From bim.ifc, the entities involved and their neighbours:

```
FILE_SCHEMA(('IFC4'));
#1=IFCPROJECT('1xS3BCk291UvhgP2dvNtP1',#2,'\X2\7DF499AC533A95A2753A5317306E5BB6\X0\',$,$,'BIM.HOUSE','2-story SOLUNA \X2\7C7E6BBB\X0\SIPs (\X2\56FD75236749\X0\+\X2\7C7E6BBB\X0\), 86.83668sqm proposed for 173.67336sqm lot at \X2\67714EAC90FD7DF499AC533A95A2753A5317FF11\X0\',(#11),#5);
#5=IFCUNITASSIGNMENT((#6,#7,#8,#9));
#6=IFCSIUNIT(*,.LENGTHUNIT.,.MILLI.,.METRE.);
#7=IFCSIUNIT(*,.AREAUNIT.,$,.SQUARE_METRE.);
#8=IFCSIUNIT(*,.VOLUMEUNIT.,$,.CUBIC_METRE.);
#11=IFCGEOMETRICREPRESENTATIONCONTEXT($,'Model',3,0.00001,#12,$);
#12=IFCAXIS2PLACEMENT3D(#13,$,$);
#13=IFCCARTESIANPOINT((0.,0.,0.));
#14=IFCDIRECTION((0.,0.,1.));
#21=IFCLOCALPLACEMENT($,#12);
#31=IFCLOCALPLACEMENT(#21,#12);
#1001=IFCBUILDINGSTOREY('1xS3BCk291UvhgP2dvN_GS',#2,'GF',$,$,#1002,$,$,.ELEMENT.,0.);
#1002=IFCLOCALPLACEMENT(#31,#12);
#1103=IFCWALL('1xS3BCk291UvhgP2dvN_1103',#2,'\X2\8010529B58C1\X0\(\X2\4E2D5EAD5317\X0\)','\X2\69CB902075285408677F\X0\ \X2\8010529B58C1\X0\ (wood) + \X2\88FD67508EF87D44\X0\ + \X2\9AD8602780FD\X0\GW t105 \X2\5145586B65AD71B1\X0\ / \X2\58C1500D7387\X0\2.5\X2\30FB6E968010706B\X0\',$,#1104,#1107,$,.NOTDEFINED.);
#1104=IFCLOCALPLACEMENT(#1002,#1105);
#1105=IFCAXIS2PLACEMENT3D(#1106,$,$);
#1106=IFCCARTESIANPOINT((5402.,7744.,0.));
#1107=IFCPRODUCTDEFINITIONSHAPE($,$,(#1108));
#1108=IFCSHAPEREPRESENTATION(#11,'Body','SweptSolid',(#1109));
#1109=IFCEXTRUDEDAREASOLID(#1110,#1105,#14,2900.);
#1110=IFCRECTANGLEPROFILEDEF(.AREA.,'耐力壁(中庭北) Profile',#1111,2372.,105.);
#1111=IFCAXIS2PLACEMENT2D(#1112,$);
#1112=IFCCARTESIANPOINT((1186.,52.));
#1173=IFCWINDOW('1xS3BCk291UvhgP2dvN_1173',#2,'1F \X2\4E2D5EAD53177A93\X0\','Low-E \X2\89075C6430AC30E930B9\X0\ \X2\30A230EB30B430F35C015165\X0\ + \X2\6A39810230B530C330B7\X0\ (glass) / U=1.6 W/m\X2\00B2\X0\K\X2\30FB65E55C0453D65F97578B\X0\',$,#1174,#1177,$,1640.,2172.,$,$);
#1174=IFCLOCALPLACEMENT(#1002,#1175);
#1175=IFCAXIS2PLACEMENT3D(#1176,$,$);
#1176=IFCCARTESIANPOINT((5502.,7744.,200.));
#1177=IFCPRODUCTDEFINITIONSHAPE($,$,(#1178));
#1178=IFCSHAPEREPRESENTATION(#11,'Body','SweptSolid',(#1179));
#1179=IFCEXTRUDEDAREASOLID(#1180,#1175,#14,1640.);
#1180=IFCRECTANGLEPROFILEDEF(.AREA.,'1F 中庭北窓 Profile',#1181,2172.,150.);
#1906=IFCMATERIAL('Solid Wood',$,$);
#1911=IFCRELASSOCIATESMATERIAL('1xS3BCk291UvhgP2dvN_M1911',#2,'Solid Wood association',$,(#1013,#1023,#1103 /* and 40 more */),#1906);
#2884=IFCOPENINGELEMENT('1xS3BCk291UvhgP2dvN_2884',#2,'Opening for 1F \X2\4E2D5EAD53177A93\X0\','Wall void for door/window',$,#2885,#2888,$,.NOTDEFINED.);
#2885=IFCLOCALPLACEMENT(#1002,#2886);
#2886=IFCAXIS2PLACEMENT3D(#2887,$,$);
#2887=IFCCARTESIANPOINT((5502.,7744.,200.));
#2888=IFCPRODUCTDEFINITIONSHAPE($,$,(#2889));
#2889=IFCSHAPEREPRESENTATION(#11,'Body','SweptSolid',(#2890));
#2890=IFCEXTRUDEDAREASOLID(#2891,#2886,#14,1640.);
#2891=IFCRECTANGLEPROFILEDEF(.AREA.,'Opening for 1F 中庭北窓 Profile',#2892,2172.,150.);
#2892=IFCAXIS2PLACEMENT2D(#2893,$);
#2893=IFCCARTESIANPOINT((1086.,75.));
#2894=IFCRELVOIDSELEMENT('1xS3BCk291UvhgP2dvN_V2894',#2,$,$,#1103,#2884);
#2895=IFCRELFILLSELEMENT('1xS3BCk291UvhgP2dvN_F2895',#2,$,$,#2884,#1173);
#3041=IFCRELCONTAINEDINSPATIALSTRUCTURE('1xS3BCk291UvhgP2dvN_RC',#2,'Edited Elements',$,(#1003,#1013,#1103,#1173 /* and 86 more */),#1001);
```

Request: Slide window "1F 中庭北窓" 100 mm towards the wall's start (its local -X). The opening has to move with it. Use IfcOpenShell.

```python
import ifcopenshell
import ifcopenshell.api.geometry
import ifcopenshell.util.placement

model = ifcopenshell.open("bim.ifc")

window = model.by_guid("1xS3BCk291UvhgP2dvN_1173")
opening = window.FillsVoids[0].RelatingOpeningElement
wall = opening.VoidsElements[0].RelatingBuildingElement

wall_matrix = ifcopenshell.util.placement.get_local_placement(wall.ObjectPlacement)
shift = wall_matrix[:3, 0] * -100.0
before = ifcopenshell.util.placement.get_local_placement(window.ObjectPlacement)[:3, 3].copy()

# The window is not placed relative to its opening, so move both.
for product in (opening, window):
    matrix = ifcopenshell.util.placement.get_local_placement(product.ObjectPlacement)
    matrix[:3, 3] += shift
    ifcopenshell.api.geometry.edit_object_placement(model, product=product, matrix=matrix, is_si=False)

after = ifcopenshell.util.placement.get_local_placement(window.ObjectPlacement)[:3, 3]
print("window moved by", (after - before).round(3) + 0.0)

model.write("bim_rev.ifc")
```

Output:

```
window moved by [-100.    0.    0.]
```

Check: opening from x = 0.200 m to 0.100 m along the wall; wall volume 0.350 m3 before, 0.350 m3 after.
